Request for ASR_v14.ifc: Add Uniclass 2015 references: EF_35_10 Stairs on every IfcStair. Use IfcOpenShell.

First a look at what the model holds.

```python
import ifcopenshell

model = ifcopenshell.open("ASR_v14.ifc")
print(model.schema)
print("classifications:", [c.Name for c in model.by_type("IfcClassification")])
for ifc_class in ("IfcDoor", "IfcRoof", "IfcStair", "IfcWall", "IfcWindow"):
    print(ifc_class, len(model.by_type(ifc_class)))
```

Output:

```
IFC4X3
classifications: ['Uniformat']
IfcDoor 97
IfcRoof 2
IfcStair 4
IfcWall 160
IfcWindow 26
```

```python
import ifcopenshell
import ifcopenshell.api.classification

model = ifcopenshell.open("ASR_v14.ifc")

system = ifcopenshell.api.classification.add_classification(model, classification="Uniclass 2015")

codes = {
    "IfcStair": ("EF_35_10", "Stairs"),
}
for ifc_class, (code, name) in codes.items():
    products = model.by_type(ifc_class)
    ifcopenshell.api.classification.add_reference(
        model, products=products, classification=system, identification=code, name=name
    )
    print(code, len(products))

model.write("ASR_v14_v2.ifc")
```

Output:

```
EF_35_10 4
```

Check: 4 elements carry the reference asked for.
